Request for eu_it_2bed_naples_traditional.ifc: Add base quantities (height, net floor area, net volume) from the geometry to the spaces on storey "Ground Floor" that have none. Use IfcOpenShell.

First a look at what the model holds.

```python
import ifcopenshell
import ifcopenshell.util.element
import ifcopenshell.util.unit

model = ifcopenshell.open("eu_it_2bed_naples_traditional.ifc")
print(model.schema)
for unit_type in ("LENGTHUNIT", "AREAUNIT", "VOLUMEUNIT"):
    print(unit_type, ifcopenshell.util.unit.calculate_unit_scale(model, unit_type))
storey = next(s for s in model.by_type("IfcBuildingStorey") if s.Name == "Ground Floor")
spaces = [e for e in ifcopenshell.util.element.get_decomposition(storey) if e.is_a("IfcSpace")]
for e in sorted(spaces, key=lambda e: e.id()):
    print(e.id(), e.is_a(), e.Name, list(ifcopenshell.util.element.get_psets(e, qtos_only=True)), sep=" | ")
```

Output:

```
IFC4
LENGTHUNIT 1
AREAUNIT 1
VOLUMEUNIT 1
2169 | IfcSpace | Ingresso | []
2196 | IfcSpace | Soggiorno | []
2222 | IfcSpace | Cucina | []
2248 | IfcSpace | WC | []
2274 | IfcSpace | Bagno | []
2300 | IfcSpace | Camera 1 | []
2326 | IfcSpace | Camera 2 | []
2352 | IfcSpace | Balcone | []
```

```python
import ifcopenshell
import ifcopenshell.api.pset
import ifcopenshell.geom
import ifcopenshell.util.element
import ifcopenshell.util.shape
import ifcopenshell.util.unit

model = ifcopenshell.open("eu_it_2bed_naples_traditional.ifc")
unit_scale = ifcopenshell.util.unit.calculate_unit_scale(model)
area_scale = ifcopenshell.util.unit.calculate_unit_scale(model, "AREAUNIT")
volume_scale = ifcopenshell.util.unit.calculate_unit_scale(model, "VOLUMEUNIT")
settings = ifcopenshell.geom.settings()

storey = next(s for s in model.by_type("IfcBuildingStorey") if s.Name == "Ground Floor")
spaces = [e for e in ifcopenshell.util.element.get_decomposition(storey) if e.is_a("IfcSpace")]

for e in sorted(spaces, key=lambda e: e.id()):
    if ifcopenshell.util.element.get_psets(e, qtos_only=True, should_inherit=False):
        continue
    # Geometry comes back in metres, in the element's own axes.
    shape = ifcopenshell.geom.create_shape(settings, e)
    values = {
        "Height": ifcopenshell.util.shape.get_z(shape.geometry) / unit_scale,
        "NetFloorArea": ifcopenshell.util.shape.get_footprint_area(shape.geometry) / area_scale,
        "NetVolume": ifcopenshell.util.shape.get_volume(shape.geometry) / volume_scale,
    }
    qto = ifcopenshell.api.pset.add_qto(model, product=e, name="Qto_SpaceBaseQuantities")
    ifcopenshell.api.pset.edit_qto(model, qto=qto, properties=values)
    print(e.id(), {k: round(v, 3) for k, v in values.items()})

model.write("eu_it_2bed_naples_traditional_rev.ifc")
```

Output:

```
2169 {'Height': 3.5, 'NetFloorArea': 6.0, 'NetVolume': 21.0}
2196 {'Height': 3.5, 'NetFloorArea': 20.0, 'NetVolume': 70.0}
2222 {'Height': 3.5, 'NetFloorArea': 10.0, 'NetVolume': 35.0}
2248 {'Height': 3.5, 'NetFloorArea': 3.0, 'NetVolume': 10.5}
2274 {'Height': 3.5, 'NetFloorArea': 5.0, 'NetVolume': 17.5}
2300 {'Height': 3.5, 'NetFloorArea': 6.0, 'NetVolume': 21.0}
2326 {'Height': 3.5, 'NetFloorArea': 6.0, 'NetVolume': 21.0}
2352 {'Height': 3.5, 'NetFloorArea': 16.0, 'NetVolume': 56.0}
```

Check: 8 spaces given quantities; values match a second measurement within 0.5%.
